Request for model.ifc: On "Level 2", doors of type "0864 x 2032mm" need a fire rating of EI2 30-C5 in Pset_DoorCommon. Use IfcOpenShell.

First a look at what the model holds.

```python
import ifcopenshell
import ifcopenshell.util.element

model = ifcopenshell.open("model.ifc")
print(model.schema)
storey = next(s for s in model.by_type("IfcBuildingStorey") if s.Name == "Level 2")
doors = [e for e in ifcopenshell.util.element.get_decomposition(storey) if e.is_a("IfcDoor")]
seen = {}
for e in doors:
    element_type = ifcopenshell.util.element.get_type(e)
    key = (element_type.Name if element_type != e and element_type else None, ifcopenshell.util.element.get_pset(e, "Pset_DoorCommon", "FireRating"))
    seen[key] = seen.get(key, 0) + 1
for (name, value), count in sorted(seen.items(), key=str):
    print(count, "x", name, "|", value)
```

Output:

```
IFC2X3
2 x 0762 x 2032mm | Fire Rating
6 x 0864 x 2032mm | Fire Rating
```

```python
import ifcopenshell
import ifcopenshell.api.pset
import ifcopenshell.util.element

model = ifcopenshell.open("model.ifc")

storey = next(s for s in model.by_type("IfcBuildingStorey") if s.Name == "Level 2")
doors = [e for e in ifcopenshell.util.element.get_decomposition(storey) if e.is_a("IfcDoor")]

count = 0
for e in doors:
    element_type = ifcopenshell.util.element.get_type(e)
    if element_type in (None, e) or element_type.Name != "0864 x 2032mm":
        continue
    # add_pset returns the element's existing set when there is one.
    pset = ifcopenshell.api.pset.add_pset(model, product=e, name="Pset_DoorCommon")
    ifcopenshell.api.pset.edit_pset(model, pset=pset, properties={"FireRating": "EI2 30-C5"})
    count += 1

print(count, "doors updated")

model.write("model_edited.ifc")
```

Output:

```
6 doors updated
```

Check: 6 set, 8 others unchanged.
